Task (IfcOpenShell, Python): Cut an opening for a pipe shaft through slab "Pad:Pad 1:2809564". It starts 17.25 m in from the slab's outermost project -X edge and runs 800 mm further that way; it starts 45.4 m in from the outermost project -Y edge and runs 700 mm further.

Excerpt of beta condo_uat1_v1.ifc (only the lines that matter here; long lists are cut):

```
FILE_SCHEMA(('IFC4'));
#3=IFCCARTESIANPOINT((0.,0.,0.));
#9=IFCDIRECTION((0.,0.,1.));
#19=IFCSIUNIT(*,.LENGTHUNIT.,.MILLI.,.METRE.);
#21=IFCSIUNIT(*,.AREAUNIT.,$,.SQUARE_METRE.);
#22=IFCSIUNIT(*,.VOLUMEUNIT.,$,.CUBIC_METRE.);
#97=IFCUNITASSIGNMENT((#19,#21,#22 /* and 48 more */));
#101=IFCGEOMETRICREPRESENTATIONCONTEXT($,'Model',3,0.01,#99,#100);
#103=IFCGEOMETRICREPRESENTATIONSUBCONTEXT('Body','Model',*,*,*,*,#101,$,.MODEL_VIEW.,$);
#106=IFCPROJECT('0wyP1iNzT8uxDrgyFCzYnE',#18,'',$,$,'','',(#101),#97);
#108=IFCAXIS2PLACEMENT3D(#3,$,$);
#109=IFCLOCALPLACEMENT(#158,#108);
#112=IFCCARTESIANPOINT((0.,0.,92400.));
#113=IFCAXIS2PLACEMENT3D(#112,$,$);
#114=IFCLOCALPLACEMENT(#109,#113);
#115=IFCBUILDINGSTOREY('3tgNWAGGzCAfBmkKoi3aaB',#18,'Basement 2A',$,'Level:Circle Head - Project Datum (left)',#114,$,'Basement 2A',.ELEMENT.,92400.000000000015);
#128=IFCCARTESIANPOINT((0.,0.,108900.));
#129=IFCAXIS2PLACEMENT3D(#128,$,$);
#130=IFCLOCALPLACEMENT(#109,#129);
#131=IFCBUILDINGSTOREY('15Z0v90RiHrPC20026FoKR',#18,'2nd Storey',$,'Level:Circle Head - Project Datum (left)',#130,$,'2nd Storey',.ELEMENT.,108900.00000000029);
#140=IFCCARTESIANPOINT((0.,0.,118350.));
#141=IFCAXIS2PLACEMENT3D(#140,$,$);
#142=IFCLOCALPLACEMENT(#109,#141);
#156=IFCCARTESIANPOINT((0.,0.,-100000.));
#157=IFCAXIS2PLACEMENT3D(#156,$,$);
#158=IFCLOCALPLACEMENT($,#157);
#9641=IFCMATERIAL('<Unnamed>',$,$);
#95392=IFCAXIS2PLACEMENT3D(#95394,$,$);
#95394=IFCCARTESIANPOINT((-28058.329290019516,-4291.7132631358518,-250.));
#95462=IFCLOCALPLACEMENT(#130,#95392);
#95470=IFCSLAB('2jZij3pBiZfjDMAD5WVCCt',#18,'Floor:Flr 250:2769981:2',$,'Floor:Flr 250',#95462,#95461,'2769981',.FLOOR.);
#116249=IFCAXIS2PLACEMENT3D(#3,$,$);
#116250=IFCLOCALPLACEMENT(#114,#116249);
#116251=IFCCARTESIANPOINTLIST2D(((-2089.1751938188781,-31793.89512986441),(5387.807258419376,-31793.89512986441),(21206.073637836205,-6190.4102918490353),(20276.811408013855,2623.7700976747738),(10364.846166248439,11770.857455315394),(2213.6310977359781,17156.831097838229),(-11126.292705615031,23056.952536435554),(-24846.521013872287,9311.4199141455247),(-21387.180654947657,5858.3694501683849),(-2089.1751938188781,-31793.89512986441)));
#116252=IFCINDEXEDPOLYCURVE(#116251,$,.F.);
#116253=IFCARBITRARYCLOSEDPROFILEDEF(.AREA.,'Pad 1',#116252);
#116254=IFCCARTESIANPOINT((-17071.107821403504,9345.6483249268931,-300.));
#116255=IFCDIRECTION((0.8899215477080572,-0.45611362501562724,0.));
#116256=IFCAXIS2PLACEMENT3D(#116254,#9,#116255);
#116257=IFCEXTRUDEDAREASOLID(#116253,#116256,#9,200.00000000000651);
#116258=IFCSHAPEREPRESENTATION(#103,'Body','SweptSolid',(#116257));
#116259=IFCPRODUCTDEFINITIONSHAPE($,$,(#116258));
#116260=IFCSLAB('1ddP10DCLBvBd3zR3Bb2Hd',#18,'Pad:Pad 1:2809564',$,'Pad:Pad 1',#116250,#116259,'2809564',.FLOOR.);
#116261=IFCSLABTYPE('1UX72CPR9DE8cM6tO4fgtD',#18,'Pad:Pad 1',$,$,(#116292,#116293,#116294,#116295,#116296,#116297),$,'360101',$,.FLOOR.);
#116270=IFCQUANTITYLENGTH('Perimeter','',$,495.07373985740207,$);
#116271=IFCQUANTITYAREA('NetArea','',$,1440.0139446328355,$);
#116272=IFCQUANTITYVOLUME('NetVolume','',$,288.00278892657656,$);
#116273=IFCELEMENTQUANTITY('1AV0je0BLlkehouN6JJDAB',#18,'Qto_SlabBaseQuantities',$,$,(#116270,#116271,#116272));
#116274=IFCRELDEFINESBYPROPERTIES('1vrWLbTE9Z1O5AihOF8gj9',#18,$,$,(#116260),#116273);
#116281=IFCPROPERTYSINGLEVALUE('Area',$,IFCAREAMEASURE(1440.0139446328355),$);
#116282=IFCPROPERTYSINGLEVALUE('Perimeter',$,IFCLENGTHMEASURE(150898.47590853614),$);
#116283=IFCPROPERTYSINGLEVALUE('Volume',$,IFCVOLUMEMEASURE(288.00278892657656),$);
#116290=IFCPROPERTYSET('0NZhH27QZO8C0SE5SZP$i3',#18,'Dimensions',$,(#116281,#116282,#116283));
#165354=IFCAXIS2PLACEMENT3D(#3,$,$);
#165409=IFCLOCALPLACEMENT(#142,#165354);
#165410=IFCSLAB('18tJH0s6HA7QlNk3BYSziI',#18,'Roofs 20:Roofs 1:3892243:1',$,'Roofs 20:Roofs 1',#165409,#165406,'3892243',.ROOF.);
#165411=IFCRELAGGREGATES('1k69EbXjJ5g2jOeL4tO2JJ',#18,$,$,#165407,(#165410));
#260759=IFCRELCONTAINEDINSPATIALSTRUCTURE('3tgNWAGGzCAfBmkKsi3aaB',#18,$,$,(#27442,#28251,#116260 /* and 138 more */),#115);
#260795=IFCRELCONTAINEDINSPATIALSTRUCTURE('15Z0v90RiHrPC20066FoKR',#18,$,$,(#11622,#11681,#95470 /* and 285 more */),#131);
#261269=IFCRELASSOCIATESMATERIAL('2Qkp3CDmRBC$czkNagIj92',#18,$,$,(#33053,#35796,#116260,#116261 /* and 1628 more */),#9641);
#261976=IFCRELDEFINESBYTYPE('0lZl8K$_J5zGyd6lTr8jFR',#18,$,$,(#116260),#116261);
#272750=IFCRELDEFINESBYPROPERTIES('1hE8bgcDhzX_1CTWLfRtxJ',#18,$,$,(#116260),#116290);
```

```python
import numpy as np
import ifcopenshell
import ifcopenshell.api.feature
import ifcopenshell.api.geometry
import ifcopenshell.api.pset
import ifcopenshell.api.root
import ifcopenshell.geom
import ifcopenshell.util.element
import ifcopenshell.util.placement
import ifcopenshell.util.representation
import ifcopenshell.util.shape
import ifcopenshell.util.unit

model = ifcopenshell.open("beta condo_uat1_v1.ifc")
unit_scale = ifcopenshell.util.unit.calculate_unit_scale(model)
area_scale = ifcopenshell.util.unit.calculate_unit_scale(model, "AREAUNIT")
volume_scale = ifcopenshell.util.unit.calculate_unit_scale(model, "VOLUMEUNIT")
settings = ifcopenshell.geom.settings()


def volume(element):
    """Net volume in cubic metres, openings subtracted."""
    shape = ifcopenshell.geom.create_shape(settings, element)
    return ifcopenshell.util.shape.get_volume(shape.geometry)


slab = model.by_id(116260)
before = volume(slab)

# Extent in the slab's own axes, in metres. The edges named are its -X and -Y sides.
slab_shape = ifcopenshell.geom.create_shape(settings, slab)
vertices = ifcopenshell.util.shape.get_vertices(slab_shape.geometry)
x_min, y_min, bottom = vertices.min(axis=0)
top = vertices[:, 2].max()

opening = ifcopenshell.api.root.create_entity(model, ifc_class="IfcOpeningElement", name="Pipe shaft opening", predefined_type="OPENING")
context = ifcopenshell.util.representation.get_context(model, "Model", "Body", "MODEL_VIEW")
width, depth = 0.8, 0.7
outline = [(0.0, 0.0), (width, 0.0), (width, depth), (0.0, depth), (0.0, 0.0)]
# Overshoot both faces by 50 mm so the cut is clean.
shape = ifcopenshell.api.geometry.add_slab_representation(
    model, context=context, depth=top - bottom + 0.1, polyline=outline
)
ifcopenshell.api.geometry.assign_representation(model, product=opening, representation=shape)

matrix = ifcopenshell.util.placement.get_local_placement(slab.ObjectPlacement)
matrix[:, 3] = matrix @ np.append(np.array([x_min + 17.25, y_min + 45.4, bottom - 0.05]) / unit_scale, 1.0)
ifcopenshell.api.geometry.edit_object_placement(model, product=opening, matrix=matrix, is_si=False)
ifcopenshell.api.feature.add_feature(model, feature=opening, element=slab)

after = volume(slab)

# Update the slab's stored quantities.
qto = model.by_id(ifcopenshell.util.element.get_pset(slab, "Qto_SlabBaseQuantities", should_inherit=False)["id"])
ifcopenshell.api.pset.edit_qto(model, qto=qto, properties={
    "NetArea": after / (top - bottom) / area_scale,
    "NetVolume": after / volume_scale,
})
pset = model.by_id(ifcopenshell.util.element.get_pset(slab, "Dimensions", should_inherit=False)["id"])
ifcopenshell.api.pset.edit_pset(model, pset=pset, properties={
    "Area": model.create_entity("IfcAreaMeasure", after / (top - bottom) / area_scale),
    "Volume": model.create_entity("IfcVolumeMeasure", after / volume_scale),
})

print(f"slab volume {before:.3f} -> {after:.3f} m3")

model.write("beta condo_uat1_v1-out.ifc")
```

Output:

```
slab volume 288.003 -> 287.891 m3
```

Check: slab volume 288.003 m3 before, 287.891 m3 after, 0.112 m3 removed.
